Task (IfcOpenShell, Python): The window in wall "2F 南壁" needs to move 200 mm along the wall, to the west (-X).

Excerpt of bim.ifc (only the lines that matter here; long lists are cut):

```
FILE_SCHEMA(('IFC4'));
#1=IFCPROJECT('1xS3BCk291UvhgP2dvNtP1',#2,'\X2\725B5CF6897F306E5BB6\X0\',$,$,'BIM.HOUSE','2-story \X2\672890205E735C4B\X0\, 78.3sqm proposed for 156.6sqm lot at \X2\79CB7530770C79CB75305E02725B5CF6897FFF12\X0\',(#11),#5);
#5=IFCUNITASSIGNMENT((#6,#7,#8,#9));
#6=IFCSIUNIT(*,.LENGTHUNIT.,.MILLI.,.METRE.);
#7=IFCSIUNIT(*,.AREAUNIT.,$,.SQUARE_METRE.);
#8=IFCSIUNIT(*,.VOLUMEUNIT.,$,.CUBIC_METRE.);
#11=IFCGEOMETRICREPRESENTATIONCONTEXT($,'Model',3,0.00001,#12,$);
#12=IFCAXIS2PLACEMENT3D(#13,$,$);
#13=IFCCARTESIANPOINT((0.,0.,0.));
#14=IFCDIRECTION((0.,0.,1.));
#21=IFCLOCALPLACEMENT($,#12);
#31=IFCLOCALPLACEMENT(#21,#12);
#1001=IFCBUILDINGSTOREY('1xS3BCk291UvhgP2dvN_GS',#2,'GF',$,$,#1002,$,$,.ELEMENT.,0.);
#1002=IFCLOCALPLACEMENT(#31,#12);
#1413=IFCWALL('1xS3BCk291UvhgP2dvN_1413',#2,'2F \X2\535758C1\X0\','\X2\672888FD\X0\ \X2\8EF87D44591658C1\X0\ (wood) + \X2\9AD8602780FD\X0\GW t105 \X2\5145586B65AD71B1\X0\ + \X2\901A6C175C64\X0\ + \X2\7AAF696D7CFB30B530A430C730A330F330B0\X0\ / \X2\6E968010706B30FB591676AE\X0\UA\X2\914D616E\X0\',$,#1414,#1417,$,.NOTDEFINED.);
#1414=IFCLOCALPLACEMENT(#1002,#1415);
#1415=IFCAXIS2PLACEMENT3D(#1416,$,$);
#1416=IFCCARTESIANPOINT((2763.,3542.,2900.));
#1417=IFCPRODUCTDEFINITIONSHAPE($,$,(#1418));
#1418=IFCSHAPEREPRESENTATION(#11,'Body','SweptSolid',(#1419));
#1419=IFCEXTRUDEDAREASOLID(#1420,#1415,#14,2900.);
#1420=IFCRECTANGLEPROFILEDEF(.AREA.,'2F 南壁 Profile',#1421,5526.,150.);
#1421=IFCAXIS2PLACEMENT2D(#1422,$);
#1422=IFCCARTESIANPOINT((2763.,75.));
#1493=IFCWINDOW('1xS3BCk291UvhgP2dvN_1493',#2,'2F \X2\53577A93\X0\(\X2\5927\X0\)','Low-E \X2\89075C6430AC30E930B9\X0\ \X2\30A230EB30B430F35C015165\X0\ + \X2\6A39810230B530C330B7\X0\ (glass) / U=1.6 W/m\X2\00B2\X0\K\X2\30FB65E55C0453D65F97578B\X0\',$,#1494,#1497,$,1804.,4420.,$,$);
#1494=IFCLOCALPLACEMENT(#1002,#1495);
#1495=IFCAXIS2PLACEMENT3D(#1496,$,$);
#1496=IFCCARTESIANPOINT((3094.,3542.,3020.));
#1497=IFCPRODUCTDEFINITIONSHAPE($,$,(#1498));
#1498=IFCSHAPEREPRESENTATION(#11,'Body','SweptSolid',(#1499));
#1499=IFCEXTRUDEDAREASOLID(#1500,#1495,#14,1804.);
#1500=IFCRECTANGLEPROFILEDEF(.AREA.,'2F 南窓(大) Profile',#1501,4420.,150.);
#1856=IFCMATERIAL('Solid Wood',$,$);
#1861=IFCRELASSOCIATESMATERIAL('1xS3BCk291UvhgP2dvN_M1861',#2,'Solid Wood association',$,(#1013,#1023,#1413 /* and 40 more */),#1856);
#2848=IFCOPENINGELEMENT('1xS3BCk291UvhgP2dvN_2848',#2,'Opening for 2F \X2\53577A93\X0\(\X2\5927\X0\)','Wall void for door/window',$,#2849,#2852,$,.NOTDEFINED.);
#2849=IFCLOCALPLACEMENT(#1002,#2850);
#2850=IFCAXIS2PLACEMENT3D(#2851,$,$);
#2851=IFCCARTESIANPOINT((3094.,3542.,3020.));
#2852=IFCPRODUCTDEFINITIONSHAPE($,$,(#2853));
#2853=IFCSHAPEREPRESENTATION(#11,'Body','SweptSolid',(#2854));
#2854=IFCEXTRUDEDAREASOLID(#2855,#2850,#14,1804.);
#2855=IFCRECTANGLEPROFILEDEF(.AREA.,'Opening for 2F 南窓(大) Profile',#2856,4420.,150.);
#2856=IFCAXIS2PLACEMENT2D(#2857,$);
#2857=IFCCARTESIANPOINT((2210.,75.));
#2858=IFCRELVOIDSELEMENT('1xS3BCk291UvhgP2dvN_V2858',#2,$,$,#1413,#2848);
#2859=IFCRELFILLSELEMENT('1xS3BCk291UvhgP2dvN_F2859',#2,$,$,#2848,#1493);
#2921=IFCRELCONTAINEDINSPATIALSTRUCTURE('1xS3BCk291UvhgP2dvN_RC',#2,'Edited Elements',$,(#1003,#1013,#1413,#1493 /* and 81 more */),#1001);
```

```python
import ifcopenshell
import ifcopenshell.api.geometry
import ifcopenshell.util.placement

model = ifcopenshell.open("bim.ifc")

window = model.by_id(1493)
opening = window.FillsVoids[0].RelatingOpeningElement
wall = opening.VoidsElements[0].RelatingBuildingElement

wall_matrix = ifcopenshell.util.placement.get_local_placement(wall.ObjectPlacement)
shift = wall_matrix[:3, 0] * -200.0
before = ifcopenshell.util.placement.get_local_placement(window.ObjectPlacement)[:3, 3].copy()

# The window is not placed relative to its opening, so move both.
for product in (opening, window):
    matrix = ifcopenshell.util.placement.get_local_placement(product.ObjectPlacement)
    matrix[:3, 3] += shift
    ifcopenshell.api.geometry.edit_object_placement(model, product=product, matrix=matrix, is_si=False)

after = ifcopenshell.util.placement.get_local_placement(window.ObjectPlacement)[:3, 3]
print("window moved by", (after - before).round(3) + 0.0)

model.write("bim_updated.ifc")
```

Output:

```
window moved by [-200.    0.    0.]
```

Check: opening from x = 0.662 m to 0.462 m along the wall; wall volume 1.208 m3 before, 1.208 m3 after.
